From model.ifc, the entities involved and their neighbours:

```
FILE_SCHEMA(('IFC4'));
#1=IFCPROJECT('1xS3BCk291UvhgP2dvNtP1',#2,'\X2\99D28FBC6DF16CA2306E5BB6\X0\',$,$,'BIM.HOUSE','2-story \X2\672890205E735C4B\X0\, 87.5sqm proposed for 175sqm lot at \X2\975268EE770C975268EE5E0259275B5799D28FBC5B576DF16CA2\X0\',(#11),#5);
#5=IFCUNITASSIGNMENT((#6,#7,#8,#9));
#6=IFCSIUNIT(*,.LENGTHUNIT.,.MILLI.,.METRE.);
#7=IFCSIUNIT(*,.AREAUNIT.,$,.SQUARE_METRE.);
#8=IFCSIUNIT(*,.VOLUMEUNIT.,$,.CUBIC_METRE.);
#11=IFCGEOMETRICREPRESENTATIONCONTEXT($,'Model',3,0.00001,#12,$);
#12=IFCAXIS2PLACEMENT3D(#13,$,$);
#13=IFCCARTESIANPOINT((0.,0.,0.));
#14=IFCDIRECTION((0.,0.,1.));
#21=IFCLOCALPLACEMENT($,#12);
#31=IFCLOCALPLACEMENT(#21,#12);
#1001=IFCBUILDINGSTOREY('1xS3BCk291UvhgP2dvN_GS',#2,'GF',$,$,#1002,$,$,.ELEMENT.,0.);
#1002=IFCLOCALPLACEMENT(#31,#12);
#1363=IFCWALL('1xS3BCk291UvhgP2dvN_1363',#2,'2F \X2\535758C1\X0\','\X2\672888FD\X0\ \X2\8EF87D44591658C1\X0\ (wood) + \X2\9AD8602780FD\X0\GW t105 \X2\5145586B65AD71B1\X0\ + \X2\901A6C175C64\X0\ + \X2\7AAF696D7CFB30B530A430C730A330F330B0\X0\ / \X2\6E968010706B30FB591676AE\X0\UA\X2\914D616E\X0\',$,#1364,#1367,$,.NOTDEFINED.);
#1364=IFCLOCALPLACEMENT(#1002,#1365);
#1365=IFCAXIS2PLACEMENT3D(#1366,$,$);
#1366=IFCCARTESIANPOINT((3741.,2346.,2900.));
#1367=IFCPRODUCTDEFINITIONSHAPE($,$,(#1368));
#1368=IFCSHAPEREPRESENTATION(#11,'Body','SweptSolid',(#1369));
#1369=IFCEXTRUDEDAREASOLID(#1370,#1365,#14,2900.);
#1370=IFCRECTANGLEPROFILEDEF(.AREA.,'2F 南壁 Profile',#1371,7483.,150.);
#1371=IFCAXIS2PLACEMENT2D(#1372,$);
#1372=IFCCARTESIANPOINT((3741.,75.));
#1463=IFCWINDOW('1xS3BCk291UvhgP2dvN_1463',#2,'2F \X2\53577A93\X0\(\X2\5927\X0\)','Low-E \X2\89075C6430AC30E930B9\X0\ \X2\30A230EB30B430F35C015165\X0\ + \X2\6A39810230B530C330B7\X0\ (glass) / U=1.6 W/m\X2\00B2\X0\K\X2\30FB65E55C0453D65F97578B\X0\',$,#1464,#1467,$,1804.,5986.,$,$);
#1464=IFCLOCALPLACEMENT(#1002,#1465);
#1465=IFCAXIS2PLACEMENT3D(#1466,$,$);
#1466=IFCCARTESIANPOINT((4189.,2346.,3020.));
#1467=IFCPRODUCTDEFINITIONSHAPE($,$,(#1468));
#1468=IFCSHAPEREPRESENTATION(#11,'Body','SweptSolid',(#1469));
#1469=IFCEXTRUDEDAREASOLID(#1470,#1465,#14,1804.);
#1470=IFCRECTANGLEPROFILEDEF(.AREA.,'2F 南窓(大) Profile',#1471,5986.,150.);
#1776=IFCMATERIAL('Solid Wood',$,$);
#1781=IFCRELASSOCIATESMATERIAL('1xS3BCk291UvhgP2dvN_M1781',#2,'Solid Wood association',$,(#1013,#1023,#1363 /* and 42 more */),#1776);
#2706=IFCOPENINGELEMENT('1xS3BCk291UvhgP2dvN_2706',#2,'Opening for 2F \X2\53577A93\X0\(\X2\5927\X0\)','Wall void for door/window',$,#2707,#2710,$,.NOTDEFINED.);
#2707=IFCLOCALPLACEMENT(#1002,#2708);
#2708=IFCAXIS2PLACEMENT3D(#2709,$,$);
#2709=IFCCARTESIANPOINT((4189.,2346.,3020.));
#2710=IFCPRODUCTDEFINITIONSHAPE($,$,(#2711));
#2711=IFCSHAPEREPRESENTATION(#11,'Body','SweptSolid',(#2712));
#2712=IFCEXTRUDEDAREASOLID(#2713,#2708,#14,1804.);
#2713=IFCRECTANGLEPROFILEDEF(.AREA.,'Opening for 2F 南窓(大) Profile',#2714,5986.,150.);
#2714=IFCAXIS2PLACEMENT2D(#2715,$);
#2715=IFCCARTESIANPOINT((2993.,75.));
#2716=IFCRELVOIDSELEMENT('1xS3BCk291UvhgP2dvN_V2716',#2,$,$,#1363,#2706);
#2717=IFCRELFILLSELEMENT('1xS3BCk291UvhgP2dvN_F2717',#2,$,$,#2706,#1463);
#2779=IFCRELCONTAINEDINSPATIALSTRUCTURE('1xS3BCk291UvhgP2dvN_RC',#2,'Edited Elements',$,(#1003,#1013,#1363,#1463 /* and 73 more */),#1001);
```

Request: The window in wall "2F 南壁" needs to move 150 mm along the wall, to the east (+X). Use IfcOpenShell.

```python
import ifcopenshell
import ifcopenshell.api.geometry
import ifcopenshell.util.placement
import ifcopenshell.util.unit

model = ifcopenshell.open("model.ifc")
unit_scale = ifcopenshell.util.unit.calculate_unit_scale(model)

window = model.by_guid("1xS3BCk291UvhgP2dvN_1463")
opening = window.FillsVoids[0].RelatingOpeningElement
wall = opening.VoidsElements[0].RelatingBuildingElement

wall_matrix = ifcopenshell.util.placement.get_local_placement(wall.ObjectPlacement)
shift = wall_matrix[:3, 0] * 0.15 / unit_scale
before = ifcopenshell.util.placement.get_local_placement(window.ObjectPlacement)[:3, 3].copy()

# The window is not placed relative to its opening, so move both.
for product in (opening, window):
    matrix = ifcopenshell.util.placement.get_local_placement(product.ObjectPlacement)
    matrix[:3, 3] += shift
    ifcopenshell.api.geometry.edit_object_placement(model, product=product, matrix=matrix, is_si=False)

after = ifcopenshell.util.placement.get_local_placement(window.ObjectPlacement)[:3, 3]
print("window moved by", (after - before).round(3) + 0.0)

model.write("model_rev.ifc")
```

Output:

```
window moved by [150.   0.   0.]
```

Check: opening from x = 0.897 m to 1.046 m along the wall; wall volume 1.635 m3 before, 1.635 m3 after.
